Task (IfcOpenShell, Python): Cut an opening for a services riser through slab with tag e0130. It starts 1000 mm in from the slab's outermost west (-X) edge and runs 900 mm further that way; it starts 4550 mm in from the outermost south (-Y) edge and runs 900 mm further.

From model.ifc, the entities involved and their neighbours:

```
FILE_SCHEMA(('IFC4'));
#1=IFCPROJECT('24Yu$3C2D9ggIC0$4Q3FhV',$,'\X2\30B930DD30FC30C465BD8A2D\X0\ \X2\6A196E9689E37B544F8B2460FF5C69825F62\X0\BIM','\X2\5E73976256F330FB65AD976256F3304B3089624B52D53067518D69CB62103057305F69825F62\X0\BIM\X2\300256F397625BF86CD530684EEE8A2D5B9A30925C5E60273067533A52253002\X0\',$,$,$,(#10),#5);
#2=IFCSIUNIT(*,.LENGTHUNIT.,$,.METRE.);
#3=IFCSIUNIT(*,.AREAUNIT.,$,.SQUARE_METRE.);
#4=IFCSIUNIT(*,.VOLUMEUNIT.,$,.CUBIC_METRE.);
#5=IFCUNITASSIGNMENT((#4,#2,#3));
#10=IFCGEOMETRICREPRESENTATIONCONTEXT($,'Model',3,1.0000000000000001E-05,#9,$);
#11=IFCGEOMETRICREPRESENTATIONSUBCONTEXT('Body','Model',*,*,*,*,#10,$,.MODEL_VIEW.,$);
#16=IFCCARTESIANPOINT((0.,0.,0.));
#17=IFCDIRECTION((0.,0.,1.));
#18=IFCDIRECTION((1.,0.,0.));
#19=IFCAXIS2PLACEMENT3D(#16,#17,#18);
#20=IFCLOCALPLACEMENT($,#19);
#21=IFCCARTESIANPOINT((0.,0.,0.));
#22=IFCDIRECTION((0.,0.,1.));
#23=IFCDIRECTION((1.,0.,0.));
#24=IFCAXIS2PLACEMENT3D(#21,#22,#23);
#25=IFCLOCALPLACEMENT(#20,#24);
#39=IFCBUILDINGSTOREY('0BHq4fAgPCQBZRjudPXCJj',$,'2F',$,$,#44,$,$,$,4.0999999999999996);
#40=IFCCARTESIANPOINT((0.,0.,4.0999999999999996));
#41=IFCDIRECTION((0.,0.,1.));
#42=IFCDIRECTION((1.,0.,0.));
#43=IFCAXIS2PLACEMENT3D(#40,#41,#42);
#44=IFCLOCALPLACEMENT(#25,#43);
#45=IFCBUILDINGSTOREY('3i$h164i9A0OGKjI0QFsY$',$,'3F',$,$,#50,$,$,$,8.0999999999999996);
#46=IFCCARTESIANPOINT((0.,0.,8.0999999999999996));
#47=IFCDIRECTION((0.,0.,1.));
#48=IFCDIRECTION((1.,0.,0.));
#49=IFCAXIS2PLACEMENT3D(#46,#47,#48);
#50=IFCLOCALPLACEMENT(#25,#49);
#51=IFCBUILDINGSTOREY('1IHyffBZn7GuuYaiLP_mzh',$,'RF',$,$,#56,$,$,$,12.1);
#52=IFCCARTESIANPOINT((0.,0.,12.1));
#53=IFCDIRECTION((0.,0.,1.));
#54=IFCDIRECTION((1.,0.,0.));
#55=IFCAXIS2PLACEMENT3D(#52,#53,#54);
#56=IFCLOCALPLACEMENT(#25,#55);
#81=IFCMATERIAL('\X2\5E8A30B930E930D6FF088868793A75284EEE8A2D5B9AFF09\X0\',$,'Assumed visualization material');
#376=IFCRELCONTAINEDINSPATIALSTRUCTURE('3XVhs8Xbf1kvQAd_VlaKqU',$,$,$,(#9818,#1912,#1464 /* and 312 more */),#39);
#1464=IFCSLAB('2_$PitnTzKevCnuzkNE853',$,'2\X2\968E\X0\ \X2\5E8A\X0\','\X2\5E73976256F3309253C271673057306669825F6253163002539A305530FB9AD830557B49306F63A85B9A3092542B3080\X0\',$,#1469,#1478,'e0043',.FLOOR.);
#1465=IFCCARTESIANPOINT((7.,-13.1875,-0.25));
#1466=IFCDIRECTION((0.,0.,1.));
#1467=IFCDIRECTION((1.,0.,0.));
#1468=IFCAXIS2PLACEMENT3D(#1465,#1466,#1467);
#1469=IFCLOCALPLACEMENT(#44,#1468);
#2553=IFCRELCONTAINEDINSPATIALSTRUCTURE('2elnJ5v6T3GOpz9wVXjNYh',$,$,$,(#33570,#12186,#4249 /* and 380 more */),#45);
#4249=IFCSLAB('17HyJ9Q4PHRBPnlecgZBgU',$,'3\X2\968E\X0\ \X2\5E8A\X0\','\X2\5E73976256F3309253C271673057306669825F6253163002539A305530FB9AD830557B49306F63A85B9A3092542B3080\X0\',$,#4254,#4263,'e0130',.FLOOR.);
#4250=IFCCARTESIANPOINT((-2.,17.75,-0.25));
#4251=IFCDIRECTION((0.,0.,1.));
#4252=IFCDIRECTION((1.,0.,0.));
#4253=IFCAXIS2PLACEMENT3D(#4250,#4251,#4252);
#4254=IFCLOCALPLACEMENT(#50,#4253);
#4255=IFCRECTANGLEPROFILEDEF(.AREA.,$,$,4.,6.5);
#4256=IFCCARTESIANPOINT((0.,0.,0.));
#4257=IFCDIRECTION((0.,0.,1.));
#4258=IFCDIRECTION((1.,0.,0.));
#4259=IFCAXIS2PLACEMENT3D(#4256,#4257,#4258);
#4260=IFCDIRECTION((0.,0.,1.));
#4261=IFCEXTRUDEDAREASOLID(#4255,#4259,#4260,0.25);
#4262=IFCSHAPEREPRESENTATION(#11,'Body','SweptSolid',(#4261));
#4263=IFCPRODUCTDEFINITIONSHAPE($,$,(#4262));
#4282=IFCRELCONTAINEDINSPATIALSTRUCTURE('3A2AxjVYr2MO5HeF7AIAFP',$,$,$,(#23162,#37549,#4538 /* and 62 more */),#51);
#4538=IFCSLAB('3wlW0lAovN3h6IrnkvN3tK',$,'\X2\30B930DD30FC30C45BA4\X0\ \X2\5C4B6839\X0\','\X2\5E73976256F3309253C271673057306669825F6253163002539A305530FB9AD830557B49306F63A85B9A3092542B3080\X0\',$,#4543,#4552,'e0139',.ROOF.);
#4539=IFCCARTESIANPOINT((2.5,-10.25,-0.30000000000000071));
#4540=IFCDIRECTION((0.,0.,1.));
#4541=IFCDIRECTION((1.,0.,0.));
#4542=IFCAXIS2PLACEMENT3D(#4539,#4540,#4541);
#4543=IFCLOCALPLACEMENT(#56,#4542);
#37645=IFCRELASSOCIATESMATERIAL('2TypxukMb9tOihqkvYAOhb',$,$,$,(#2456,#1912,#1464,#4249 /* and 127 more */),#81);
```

```python
import numpy as np
import ifcopenshell
import ifcopenshell.api.feature
import ifcopenshell.api.geometry
import ifcopenshell.api.root
import ifcopenshell.geom
import ifcopenshell.util.placement
import ifcopenshell.util.representation
import ifcopenshell.util.shape
import ifcopenshell.util.unit

model = ifcopenshell.open("model.ifc")
unit_scale = ifcopenshell.util.unit.calculate_unit_scale(model)
settings = ifcopenshell.geom.settings()


def volume(element):
    """Net volume in cubic metres, openings subtracted."""
    shape = ifcopenshell.geom.create_shape(settings, element)
    return ifcopenshell.util.shape.get_volume(shape.geometry)


slab = model.by_guid("17HyJ9Q4PHRBPnlecgZBgU")
before = volume(slab)

# Extent in the slab's own axes, in metres. The edges named are its -X and -Y sides.
slab_shape = ifcopenshell.geom.create_shape(settings, slab)
vertices = ifcopenshell.util.shape.get_vertices(slab_shape.geometry)
x_min, y_min, bottom = vertices.min(axis=0)
top = vertices[:, 2].max()

opening = ifcopenshell.api.root.create_entity(model, ifc_class="IfcOpeningElement", name="Services riser opening", predefined_type="OPENING")
context = ifcopenshell.util.representation.get_context(model, "Model", "Body", "MODEL_VIEW")
width, depth = 0.9, 0.9
outline = [(0.0, 0.0), (width, 0.0), (width, depth), (0.0, depth), (0.0, 0.0)]
# Overshoot both faces by 50 mm so the cut is clean.
shape = ifcopenshell.api.geometry.add_slab_representation(
    model, context=context, depth=top - bottom + 0.1, polyline=outline
)
ifcopenshell.api.geometry.assign_representation(model, product=opening, representation=shape)

matrix = ifcopenshell.util.placement.get_local_placement(slab.ObjectPlacement)
matrix[:, 3] = matrix @ np.append(np.array([x_min + 1, y_min + 4.55, bottom - 0.05]) / unit_scale, 1.0)
ifcopenshell.api.geometry.edit_object_placement(model, product=opening, matrix=matrix, is_si=False)
ifcopenshell.api.feature.add_feature(model, feature=opening, element=slab)

after = volume(slab)

print(f"slab volume {before:.3f} -> {after:.3f} m3")

model.write("model_rev.ifc")
```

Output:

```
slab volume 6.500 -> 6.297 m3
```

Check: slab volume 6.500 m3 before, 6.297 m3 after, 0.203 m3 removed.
